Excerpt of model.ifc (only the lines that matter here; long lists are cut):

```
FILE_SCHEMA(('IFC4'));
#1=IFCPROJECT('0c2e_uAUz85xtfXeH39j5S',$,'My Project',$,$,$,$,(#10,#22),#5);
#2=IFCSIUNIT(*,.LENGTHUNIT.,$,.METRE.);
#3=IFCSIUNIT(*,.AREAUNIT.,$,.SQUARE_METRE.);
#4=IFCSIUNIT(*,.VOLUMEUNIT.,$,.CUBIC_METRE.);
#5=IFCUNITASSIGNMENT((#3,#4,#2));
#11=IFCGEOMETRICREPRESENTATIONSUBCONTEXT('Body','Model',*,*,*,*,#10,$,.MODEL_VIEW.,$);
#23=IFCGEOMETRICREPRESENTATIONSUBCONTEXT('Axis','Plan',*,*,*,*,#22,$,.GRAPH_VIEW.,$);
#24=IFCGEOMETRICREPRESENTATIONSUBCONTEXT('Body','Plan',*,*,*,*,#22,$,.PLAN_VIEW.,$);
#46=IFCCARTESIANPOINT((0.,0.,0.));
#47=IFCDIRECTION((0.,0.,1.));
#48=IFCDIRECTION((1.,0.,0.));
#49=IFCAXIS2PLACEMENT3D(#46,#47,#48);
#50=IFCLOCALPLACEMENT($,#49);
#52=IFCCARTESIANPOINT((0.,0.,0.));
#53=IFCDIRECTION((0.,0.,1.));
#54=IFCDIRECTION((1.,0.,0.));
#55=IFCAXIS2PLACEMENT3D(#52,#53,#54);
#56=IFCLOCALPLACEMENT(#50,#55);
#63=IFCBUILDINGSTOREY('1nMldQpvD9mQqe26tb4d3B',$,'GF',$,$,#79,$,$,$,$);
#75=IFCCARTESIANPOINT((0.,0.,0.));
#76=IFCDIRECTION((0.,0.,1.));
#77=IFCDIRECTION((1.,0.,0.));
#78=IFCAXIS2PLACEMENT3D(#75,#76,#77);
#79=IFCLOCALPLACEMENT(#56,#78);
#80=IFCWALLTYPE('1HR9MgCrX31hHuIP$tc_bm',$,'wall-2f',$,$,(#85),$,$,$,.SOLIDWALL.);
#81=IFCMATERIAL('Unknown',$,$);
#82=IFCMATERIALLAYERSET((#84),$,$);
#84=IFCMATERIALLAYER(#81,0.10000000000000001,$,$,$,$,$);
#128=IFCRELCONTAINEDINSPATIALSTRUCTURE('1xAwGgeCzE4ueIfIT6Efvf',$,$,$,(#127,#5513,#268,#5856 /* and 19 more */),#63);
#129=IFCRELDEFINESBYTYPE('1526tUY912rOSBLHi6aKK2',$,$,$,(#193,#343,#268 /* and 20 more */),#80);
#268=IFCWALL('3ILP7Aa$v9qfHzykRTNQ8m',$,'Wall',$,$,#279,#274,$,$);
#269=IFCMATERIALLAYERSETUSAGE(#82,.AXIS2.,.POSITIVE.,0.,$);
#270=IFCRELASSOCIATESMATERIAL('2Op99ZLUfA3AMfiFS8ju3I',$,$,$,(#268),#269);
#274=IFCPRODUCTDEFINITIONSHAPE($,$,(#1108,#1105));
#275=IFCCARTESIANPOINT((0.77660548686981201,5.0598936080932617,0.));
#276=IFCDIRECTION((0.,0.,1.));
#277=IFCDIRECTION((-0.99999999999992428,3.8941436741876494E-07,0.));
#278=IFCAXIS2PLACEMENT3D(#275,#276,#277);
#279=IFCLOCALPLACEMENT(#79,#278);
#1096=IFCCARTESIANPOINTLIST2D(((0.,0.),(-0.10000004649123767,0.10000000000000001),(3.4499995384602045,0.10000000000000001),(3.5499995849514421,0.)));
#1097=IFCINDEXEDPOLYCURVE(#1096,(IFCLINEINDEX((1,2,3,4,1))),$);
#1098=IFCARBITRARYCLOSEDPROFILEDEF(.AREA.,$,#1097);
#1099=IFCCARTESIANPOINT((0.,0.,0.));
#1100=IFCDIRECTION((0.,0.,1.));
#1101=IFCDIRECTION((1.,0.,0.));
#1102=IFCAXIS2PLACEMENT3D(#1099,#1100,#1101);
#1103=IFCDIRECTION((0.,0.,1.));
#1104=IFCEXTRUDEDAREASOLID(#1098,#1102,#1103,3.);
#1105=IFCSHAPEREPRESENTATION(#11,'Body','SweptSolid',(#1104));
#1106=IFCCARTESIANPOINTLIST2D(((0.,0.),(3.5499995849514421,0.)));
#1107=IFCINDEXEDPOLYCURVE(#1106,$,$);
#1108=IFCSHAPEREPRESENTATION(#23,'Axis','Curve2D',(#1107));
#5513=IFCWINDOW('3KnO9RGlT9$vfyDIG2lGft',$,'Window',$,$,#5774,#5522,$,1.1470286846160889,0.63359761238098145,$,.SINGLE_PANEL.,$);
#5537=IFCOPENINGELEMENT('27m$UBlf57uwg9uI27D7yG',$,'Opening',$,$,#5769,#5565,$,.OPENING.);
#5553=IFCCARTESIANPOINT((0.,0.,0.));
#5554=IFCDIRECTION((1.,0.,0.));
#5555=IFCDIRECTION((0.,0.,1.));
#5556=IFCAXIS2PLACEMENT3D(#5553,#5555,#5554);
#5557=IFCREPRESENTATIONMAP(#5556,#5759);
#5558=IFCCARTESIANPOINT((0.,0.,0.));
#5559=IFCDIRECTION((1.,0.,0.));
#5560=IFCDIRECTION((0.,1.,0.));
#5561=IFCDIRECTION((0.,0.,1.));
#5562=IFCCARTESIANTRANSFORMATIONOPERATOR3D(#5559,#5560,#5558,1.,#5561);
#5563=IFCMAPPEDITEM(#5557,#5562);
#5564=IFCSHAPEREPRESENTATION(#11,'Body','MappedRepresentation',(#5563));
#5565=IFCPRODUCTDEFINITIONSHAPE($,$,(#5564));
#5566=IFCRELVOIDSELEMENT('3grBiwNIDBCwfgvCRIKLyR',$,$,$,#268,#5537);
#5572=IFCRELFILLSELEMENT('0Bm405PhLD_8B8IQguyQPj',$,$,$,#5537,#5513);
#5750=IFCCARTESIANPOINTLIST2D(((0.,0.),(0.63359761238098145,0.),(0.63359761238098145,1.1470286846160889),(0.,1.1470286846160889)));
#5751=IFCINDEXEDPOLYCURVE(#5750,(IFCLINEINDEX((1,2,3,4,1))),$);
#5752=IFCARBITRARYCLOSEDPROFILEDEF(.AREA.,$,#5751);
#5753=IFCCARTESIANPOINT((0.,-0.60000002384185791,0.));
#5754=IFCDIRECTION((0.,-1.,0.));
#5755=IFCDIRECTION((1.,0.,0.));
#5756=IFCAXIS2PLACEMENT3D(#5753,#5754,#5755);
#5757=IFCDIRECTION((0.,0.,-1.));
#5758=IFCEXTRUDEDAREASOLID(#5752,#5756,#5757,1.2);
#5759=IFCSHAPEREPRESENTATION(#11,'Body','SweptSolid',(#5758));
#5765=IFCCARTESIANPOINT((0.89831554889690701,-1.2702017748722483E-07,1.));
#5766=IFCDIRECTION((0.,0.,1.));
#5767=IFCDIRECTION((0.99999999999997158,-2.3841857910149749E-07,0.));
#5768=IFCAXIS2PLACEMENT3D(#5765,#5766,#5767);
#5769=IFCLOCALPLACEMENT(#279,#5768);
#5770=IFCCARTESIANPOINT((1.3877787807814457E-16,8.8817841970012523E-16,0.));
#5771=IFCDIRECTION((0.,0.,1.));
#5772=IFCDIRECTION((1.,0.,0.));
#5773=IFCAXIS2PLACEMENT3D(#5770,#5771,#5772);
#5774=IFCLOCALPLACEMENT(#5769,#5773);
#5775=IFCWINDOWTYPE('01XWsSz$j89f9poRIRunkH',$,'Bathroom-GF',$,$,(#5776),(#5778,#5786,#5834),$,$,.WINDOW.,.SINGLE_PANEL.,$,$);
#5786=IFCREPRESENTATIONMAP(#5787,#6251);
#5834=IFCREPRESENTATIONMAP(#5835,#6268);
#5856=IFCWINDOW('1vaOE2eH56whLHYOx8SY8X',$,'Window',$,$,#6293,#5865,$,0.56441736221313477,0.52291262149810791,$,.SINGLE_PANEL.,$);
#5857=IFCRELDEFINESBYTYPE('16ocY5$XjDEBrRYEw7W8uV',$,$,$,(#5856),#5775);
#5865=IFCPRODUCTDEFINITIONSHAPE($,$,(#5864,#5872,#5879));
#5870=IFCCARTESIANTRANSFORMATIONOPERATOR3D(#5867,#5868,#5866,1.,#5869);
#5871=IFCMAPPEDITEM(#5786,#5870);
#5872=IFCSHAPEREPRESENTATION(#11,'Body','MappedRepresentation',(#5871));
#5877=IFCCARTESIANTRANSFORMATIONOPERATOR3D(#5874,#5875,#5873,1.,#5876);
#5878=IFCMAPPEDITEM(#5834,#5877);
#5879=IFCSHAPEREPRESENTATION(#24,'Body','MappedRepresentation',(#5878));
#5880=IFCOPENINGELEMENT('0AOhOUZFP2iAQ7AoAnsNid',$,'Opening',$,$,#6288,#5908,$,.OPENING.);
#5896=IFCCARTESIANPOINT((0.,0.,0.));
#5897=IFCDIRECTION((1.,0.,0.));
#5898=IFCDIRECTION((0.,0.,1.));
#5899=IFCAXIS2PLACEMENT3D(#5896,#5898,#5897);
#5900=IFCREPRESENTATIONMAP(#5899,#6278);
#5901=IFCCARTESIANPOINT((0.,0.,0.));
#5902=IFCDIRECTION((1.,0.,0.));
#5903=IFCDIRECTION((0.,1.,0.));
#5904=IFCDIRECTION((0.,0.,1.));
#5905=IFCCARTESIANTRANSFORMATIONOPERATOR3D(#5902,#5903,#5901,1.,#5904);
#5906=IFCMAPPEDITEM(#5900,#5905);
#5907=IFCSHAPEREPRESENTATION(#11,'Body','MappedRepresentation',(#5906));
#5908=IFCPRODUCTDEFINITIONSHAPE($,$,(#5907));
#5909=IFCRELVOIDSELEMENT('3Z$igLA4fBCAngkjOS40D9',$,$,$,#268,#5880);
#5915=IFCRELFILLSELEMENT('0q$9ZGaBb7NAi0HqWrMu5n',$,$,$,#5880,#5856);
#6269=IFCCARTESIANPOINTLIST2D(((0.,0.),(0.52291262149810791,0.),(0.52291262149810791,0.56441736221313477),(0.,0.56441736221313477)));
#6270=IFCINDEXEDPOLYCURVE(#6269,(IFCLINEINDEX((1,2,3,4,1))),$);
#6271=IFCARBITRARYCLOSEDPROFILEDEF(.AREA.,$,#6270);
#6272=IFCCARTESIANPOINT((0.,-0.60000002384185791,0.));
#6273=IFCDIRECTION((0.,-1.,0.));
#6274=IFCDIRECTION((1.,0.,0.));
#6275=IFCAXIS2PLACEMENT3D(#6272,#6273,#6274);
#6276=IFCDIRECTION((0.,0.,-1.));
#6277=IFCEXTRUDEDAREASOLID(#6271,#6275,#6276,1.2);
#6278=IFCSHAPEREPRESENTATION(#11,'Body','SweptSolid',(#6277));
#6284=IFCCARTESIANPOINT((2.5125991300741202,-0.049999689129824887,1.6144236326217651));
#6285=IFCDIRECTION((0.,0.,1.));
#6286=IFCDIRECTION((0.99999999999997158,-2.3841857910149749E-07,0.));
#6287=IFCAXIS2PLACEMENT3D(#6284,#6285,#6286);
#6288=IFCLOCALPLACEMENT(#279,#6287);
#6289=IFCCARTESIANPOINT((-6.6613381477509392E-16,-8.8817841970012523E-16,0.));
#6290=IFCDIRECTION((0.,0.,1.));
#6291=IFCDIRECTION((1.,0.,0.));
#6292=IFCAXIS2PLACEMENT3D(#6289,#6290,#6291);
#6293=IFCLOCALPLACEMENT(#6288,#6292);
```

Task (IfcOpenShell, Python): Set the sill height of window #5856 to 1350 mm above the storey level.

```python
import numpy as np
import ifcopenshell
import ifcopenshell.api.geometry
import ifcopenshell.geom
import ifcopenshell.util.element
import ifcopenshell.util.placement
import ifcopenshell.util.shape
import ifcopenshell.util.unit

model = ifcopenshell.open("model.ifc")
unit_scale = ifcopenshell.util.unit.calculate_unit_scale(model)

window = model.by_guid("1vaOE2eH56whLHYOx8SY8X")
opening = window.FillsVoids[0].RelatingOpeningElement
storey = ifcopenshell.util.element.get_container(window, ifc_class="IfcBuildingStorey")
level = ifcopenshell.util.placement.get_local_placement(storey.ObjectPlacement)[2, 3]

# The opening's origin need not be at the sill, so measure its lowest point.
shape = ifcopenshell.geom.create_shape(ifcopenshell.geom.settings(), opening)
bottom = ifcopenshell.util.shape.get_shape_bottom_elevation(shape, shape.geometry) / unit_scale
dz = level + 1.35 / unit_scale - bottom

shift = np.array([0.0, 0.0, dz])
# The window is placed relative to its opening, so it follows when the opening moves.
matrix = ifcopenshell.util.placement.get_local_placement(opening.ObjectPlacement)
matrix[:3, 3] += shift
ifcopenshell.api.geometry.edit_object_placement(
    model, product=opening, matrix=matrix, is_si=False, should_transform_children=True
)

print(f"moved by {dz * unit_scale:+.3f} m")

model.write("model_v2.ifc")
```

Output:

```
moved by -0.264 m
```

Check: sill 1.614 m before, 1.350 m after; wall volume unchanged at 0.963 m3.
